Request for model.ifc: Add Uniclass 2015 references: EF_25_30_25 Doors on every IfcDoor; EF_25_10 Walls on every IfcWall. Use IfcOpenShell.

First a look at what the model holds.

```python
import ifcopenshell

model = ifcopenshell.open("model.ifc")
print(model.schema)
print("classifications:", [c.Name for c in model.by_type("IfcClassification")])
for ifc_class in ("IfcDoor", "IfcRoof", "IfcStair", "IfcWall", "IfcWindow"):
    print(ifc_class, len(model.by_type(ifc_class)))
```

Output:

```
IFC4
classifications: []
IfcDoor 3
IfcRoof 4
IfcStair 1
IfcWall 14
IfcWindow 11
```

```python
import ifcopenshell
import ifcopenshell.api.classification

model = ifcopenshell.open("model.ifc")

system = ifcopenshell.api.classification.add_classification(model, classification="Uniclass 2015")

codes = {
    "IfcDoor": ("EF_25_30_25", "Doors"),
    "IfcWall": ("EF_25_10", "Walls"),
}
for ifc_class, (code, name) in codes.items():
    products = model.by_type(ifc_class)
    ifcopenshell.api.classification.add_reference(
        model, products=products, classification=system, identification=code, name=name
    )
    print(code, len(products))

model.write("model_v2.ifc")
```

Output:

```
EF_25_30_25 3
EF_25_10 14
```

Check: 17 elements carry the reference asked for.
